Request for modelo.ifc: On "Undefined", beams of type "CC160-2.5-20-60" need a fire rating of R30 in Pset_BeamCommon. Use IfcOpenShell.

First a look at what the model holds.

```python
import ifcopenshell
import ifcopenshell.util.element

model = ifcopenshell.open("modelo.ifc")
print(model.schema)
storey = next(s for s in model.by_type("IfcBuildingStorey") if s.Name == "Undefined")
beams = [e for e in ifcopenshell.util.element.get_decomposition(storey) if e.is_a("IfcBeam")]
seen = {}
for e in beams:
    element_type = ifcopenshell.util.element.get_type(e)
    key = (element_type.Name if element_type != e and element_type else None, ifcopenshell.util.element.get_pset(e, "Pset_BeamCommon", "FireRating"))
    seen[key] = seen.get(key, 0) + 1
for (name, value), count in sorted(seen.items(), key=str):
    print(count, "x", name, "|", value)
```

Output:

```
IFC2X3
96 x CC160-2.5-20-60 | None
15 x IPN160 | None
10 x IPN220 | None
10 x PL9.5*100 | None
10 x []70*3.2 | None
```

```python
import ifcopenshell
import ifcopenshell.api.pset
import ifcopenshell.util.element

model = ifcopenshell.open("modelo.ifc")

storey = next(s for s in model.by_type("IfcBuildingStorey") if s.Name == "Undefined")
beams = [e for e in ifcopenshell.util.element.get_decomposition(storey) if e.is_a("IfcBeam")]

count = 0
for e in beams:
    element_type = ifcopenshell.util.element.get_type(e)
    if element_type in (None, e) or element_type.Name != "CC160-2.5-20-60":
        continue
    found = ifcopenshell.util.element.get_pset(e, "Pset_BeamCommon", should_inherit=False)
    if found:
        pset = model.by_id(found["id"])
        if len(ifcopenshell.util.element.get_elements_by_pset(pset)) > 1:
            pset = ifcopenshell.api.pset.unshare_pset(model, products=[e], pset=pset)[0]
    else:
        pset = ifcopenshell.api.pset.add_pset(model, product=e, name="Pset_BeamCommon")
    ifcopenshell.api.pset.edit_pset(model, pset=pset, properties={"FireRating": "R30"})
    count += 1

print(count, "beams updated")

model.write("modelo_v2.ifc")
```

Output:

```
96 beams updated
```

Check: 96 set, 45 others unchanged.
